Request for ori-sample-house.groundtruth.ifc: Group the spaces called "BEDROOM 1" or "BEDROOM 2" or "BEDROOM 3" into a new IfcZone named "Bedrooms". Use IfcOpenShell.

First a look at what the model holds.

```python
import ifcopenshell

model = ifcopenshell.open("ori-sample-house.groundtruth.ifc")
print(model.schema)
seen = {}
for space in model.by_type("IfcSpace"):
    seen[space.Name] = seen.get(space.Name, 0) + 1
for name, count in sorted(seen.items(), key=str):
    print(count, "x", name)
print("zones:", [z.Name for z in model.by_type("IfcZone")][:20])
```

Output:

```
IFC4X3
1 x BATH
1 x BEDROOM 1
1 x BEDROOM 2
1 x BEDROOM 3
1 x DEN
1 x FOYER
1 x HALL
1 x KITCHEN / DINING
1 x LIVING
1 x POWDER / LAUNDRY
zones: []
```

```python
import ifcopenshell
import ifcopenshell.api.group
import ifcopenshell.api.root

model = ifcopenshell.open("ori-sample-house.groundtruth.ifc")

names = {"BEDROOM 1", "BEDROOM 2", "BEDROOM 3"}
spaces = [s for s in model.by_type("IfcSpace") if s.Name in names]

zone = ifcopenshell.api.root.create_entity(model, ifc_class="IfcZone", name="Bedrooms")
ifcopenshell.api.group.assign_group(model, products=spaces, group=zone)
print(len(spaces), "spaces in", zone.Name)

model.write("ori-sample-house.groundtruth_edited.ifc")
```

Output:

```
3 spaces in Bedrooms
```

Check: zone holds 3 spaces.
